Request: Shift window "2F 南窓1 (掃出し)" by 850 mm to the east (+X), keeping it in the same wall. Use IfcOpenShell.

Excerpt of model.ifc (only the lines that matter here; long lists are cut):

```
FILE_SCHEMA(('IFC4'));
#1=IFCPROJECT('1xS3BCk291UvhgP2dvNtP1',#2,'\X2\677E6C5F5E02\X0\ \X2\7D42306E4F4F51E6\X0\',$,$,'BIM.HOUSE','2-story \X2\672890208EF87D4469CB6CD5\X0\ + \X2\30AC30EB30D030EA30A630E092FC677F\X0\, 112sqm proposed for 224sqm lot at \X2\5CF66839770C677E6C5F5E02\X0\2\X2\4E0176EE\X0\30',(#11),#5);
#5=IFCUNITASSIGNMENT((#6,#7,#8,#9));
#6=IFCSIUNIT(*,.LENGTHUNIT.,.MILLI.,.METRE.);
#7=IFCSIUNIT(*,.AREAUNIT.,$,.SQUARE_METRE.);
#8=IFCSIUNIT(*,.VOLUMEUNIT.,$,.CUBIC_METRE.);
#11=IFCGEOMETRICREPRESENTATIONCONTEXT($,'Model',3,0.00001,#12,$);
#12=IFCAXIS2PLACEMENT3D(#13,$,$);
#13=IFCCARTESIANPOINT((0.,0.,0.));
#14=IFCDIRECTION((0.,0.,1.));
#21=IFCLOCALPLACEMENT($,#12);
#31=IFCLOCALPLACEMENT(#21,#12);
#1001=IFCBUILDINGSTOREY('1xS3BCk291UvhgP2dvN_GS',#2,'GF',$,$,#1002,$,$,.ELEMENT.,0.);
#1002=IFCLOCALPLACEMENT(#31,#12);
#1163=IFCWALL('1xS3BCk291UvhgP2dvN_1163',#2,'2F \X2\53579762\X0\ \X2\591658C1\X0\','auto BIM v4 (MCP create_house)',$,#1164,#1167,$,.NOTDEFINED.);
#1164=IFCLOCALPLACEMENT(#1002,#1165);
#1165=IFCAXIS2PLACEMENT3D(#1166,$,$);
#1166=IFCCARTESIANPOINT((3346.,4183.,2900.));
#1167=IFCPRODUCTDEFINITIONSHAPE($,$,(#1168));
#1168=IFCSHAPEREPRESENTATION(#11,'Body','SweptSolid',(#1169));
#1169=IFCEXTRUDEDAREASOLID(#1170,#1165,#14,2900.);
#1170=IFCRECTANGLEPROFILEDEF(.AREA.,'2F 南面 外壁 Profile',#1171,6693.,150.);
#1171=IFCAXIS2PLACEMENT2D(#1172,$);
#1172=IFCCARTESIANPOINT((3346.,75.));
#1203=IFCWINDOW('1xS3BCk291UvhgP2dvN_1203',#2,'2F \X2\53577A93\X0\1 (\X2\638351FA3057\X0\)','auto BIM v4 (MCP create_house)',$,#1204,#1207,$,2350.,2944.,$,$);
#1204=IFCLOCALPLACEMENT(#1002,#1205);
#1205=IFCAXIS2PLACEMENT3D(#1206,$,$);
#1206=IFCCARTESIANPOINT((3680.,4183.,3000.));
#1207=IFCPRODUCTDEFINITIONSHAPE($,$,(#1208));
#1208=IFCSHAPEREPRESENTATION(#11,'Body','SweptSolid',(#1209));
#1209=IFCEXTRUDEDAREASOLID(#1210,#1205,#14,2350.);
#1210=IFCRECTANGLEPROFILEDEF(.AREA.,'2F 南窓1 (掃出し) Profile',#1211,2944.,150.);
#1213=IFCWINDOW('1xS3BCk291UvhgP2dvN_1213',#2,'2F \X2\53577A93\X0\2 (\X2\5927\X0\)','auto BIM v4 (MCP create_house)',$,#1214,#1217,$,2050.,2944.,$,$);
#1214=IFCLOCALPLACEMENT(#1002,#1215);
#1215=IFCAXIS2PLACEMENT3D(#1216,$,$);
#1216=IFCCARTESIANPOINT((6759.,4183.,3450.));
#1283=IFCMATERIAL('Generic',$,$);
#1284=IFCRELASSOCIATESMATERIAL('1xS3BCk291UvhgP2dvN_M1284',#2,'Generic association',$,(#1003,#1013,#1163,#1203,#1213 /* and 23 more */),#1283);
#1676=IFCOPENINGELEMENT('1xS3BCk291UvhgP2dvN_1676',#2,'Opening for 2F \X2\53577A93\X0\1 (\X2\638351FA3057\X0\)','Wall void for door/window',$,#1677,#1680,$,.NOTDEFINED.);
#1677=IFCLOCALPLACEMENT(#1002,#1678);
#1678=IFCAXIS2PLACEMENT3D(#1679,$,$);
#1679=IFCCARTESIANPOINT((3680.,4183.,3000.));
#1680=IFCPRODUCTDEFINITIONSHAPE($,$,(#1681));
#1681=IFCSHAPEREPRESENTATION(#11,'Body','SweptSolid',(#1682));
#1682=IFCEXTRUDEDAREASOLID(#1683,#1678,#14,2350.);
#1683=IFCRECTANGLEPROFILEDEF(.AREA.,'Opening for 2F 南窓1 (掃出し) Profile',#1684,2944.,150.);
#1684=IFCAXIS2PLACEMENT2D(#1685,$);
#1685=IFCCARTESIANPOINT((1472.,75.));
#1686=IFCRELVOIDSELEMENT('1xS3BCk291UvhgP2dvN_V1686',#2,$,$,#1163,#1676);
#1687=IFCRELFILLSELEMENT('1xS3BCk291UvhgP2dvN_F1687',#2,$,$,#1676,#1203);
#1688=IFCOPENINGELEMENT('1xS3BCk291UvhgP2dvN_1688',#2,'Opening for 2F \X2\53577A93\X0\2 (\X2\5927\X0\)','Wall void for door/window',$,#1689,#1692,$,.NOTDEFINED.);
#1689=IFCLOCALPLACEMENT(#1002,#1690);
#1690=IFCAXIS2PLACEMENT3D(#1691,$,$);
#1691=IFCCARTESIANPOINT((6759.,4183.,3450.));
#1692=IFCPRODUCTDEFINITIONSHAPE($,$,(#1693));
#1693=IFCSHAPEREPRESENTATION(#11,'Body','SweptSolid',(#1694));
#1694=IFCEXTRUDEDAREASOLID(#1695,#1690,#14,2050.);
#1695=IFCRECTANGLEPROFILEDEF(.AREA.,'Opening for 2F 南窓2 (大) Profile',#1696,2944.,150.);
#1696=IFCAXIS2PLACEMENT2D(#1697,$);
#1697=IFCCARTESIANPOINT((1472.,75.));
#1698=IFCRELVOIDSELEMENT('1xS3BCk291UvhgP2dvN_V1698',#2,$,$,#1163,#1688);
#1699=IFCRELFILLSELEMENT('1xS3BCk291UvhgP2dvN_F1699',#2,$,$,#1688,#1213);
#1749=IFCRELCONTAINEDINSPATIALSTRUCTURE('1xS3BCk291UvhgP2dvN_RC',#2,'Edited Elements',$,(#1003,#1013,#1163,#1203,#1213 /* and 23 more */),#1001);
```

```python
import ifcopenshell
import ifcopenshell.api.geometry
import ifcopenshell.util.placement

model = ifcopenshell.open("model.ifc")

window = model.by_guid("1xS3BCk291UvhgP2dvN_1203")
opening = window.FillsVoids[0].RelatingOpeningElement
wall = opening.VoidsElements[0].RelatingBuildingElement

wall_matrix = ifcopenshell.util.placement.get_local_placement(wall.ObjectPlacement)
shift = wall_matrix[:3, 0] * 850.0
before = ifcopenshell.util.placement.get_local_placement(window.ObjectPlacement)[:3, 3].copy()

# The window is not placed relative to its opening, so move both.
for product in (opening, window):
    matrix = ifcopenshell.util.placement.get_local_placement(product.ObjectPlacement)
    matrix[:3, 3] += shift
    ifcopenshell.api.geometry.edit_object_placement(model, product=product, matrix=matrix, is_si=False)

after = ifcopenshell.util.placement.get_local_placement(window.ObjectPlacement)[:3, 3]
print("window moved by", (after - before).round(3) + 0.0)

model.write("model_edited.ifc")
```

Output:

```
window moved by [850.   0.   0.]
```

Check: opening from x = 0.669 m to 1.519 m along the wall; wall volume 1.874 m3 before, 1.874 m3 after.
